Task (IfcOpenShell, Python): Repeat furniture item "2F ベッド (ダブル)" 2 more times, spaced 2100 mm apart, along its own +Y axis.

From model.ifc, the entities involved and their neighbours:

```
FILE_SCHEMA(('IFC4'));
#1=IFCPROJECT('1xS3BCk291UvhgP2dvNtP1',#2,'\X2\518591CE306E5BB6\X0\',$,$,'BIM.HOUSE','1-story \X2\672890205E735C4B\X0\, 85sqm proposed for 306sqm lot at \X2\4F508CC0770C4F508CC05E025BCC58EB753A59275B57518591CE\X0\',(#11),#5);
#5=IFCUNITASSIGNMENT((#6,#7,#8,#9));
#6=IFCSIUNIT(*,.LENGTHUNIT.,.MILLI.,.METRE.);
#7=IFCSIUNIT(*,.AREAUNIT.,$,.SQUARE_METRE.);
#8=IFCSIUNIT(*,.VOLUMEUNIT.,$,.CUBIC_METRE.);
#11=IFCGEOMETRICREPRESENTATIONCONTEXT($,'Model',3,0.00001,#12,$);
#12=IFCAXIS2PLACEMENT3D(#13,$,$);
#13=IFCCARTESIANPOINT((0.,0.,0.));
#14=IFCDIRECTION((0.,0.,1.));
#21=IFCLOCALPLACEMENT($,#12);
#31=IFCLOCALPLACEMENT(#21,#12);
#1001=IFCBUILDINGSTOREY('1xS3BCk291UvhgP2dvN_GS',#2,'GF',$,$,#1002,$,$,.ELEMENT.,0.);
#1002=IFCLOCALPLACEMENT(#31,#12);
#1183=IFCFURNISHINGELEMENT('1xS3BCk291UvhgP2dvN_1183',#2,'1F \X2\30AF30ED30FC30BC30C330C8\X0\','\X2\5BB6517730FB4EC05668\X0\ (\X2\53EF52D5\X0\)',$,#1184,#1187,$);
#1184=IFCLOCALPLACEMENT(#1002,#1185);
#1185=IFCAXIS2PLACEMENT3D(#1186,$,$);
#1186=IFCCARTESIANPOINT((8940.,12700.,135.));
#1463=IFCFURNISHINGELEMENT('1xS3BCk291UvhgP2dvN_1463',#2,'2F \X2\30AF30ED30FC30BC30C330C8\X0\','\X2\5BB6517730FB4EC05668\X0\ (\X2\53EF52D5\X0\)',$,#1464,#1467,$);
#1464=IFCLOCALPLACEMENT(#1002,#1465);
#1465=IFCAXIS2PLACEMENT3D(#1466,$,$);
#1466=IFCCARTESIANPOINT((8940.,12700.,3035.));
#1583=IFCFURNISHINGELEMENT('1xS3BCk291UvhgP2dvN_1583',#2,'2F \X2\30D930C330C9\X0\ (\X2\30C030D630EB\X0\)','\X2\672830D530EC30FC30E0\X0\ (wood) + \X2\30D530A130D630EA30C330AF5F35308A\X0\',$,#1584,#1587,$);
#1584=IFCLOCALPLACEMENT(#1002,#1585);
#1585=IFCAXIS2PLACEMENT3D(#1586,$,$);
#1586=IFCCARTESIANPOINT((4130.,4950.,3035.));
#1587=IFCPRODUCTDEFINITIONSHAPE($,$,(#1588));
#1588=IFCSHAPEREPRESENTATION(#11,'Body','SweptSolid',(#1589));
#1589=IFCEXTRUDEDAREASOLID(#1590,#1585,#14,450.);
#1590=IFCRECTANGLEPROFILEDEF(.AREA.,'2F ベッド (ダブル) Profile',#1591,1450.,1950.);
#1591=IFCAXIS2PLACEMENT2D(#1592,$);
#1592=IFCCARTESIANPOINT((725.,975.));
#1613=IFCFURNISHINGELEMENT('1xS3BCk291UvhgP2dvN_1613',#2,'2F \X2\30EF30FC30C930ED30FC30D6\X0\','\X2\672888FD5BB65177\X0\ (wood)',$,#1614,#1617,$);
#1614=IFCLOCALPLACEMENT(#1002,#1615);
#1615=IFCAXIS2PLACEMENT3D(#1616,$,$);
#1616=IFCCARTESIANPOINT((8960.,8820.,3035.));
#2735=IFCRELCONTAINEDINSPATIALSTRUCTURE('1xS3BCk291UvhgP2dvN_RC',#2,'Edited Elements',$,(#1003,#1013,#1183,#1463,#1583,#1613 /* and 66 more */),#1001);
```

```python
import ifcopenshell
import ifcopenshell.api.geometry
import ifcopenshell.api.root
import ifcopenshell.util.element
import ifcopenshell.util.placement

model = ifcopenshell.open("model.ifc")


def reuse_history(source, copy):
    """copy_class also copies each property set's owner history, people and application; keep the originals."""
    for rel in copy.IsDefinedBy:
        if rel.is_a("IfcRelDefinesByProperties") and (history := rel.RelatingPropertyDefinition.OwnerHistory):
            rel.RelatingPropertyDefinition.OwnerHistory = source.OwnerHistory
            ifcopenshell.util.element.remove_deep2(model, history)


source = model.by_guid("1xS3BCk291UvhgP2dvN_1583")
base = ifcopenshell.util.placement.get_local_placement(source.ObjectPlacement)
step = base[:3, 1] * 2100.0

for i in range(1, 3):
    copy = ifcopenshell.api.root.copy_class(model, product=source)
    copy.Representation = ifcopenshell.util.element.copy_deep(
        model, source.Representation, exclude=["IfcGeometricRepresentationContext", "IfcRepresentationMap"]
    )
    reuse_history(source, copy)
    matrix = base.copy()
    matrix[:3, 3] += i * step
    print("added at", matrix[:3, 3].round(3) + 0.0)
    ifcopenshell.api.geometry.edit_object_placement(model, product=copy, matrix=matrix, is_si=False)

model.write("model_rev.ifc")
```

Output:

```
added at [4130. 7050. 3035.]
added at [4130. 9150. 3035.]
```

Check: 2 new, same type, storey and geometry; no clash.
